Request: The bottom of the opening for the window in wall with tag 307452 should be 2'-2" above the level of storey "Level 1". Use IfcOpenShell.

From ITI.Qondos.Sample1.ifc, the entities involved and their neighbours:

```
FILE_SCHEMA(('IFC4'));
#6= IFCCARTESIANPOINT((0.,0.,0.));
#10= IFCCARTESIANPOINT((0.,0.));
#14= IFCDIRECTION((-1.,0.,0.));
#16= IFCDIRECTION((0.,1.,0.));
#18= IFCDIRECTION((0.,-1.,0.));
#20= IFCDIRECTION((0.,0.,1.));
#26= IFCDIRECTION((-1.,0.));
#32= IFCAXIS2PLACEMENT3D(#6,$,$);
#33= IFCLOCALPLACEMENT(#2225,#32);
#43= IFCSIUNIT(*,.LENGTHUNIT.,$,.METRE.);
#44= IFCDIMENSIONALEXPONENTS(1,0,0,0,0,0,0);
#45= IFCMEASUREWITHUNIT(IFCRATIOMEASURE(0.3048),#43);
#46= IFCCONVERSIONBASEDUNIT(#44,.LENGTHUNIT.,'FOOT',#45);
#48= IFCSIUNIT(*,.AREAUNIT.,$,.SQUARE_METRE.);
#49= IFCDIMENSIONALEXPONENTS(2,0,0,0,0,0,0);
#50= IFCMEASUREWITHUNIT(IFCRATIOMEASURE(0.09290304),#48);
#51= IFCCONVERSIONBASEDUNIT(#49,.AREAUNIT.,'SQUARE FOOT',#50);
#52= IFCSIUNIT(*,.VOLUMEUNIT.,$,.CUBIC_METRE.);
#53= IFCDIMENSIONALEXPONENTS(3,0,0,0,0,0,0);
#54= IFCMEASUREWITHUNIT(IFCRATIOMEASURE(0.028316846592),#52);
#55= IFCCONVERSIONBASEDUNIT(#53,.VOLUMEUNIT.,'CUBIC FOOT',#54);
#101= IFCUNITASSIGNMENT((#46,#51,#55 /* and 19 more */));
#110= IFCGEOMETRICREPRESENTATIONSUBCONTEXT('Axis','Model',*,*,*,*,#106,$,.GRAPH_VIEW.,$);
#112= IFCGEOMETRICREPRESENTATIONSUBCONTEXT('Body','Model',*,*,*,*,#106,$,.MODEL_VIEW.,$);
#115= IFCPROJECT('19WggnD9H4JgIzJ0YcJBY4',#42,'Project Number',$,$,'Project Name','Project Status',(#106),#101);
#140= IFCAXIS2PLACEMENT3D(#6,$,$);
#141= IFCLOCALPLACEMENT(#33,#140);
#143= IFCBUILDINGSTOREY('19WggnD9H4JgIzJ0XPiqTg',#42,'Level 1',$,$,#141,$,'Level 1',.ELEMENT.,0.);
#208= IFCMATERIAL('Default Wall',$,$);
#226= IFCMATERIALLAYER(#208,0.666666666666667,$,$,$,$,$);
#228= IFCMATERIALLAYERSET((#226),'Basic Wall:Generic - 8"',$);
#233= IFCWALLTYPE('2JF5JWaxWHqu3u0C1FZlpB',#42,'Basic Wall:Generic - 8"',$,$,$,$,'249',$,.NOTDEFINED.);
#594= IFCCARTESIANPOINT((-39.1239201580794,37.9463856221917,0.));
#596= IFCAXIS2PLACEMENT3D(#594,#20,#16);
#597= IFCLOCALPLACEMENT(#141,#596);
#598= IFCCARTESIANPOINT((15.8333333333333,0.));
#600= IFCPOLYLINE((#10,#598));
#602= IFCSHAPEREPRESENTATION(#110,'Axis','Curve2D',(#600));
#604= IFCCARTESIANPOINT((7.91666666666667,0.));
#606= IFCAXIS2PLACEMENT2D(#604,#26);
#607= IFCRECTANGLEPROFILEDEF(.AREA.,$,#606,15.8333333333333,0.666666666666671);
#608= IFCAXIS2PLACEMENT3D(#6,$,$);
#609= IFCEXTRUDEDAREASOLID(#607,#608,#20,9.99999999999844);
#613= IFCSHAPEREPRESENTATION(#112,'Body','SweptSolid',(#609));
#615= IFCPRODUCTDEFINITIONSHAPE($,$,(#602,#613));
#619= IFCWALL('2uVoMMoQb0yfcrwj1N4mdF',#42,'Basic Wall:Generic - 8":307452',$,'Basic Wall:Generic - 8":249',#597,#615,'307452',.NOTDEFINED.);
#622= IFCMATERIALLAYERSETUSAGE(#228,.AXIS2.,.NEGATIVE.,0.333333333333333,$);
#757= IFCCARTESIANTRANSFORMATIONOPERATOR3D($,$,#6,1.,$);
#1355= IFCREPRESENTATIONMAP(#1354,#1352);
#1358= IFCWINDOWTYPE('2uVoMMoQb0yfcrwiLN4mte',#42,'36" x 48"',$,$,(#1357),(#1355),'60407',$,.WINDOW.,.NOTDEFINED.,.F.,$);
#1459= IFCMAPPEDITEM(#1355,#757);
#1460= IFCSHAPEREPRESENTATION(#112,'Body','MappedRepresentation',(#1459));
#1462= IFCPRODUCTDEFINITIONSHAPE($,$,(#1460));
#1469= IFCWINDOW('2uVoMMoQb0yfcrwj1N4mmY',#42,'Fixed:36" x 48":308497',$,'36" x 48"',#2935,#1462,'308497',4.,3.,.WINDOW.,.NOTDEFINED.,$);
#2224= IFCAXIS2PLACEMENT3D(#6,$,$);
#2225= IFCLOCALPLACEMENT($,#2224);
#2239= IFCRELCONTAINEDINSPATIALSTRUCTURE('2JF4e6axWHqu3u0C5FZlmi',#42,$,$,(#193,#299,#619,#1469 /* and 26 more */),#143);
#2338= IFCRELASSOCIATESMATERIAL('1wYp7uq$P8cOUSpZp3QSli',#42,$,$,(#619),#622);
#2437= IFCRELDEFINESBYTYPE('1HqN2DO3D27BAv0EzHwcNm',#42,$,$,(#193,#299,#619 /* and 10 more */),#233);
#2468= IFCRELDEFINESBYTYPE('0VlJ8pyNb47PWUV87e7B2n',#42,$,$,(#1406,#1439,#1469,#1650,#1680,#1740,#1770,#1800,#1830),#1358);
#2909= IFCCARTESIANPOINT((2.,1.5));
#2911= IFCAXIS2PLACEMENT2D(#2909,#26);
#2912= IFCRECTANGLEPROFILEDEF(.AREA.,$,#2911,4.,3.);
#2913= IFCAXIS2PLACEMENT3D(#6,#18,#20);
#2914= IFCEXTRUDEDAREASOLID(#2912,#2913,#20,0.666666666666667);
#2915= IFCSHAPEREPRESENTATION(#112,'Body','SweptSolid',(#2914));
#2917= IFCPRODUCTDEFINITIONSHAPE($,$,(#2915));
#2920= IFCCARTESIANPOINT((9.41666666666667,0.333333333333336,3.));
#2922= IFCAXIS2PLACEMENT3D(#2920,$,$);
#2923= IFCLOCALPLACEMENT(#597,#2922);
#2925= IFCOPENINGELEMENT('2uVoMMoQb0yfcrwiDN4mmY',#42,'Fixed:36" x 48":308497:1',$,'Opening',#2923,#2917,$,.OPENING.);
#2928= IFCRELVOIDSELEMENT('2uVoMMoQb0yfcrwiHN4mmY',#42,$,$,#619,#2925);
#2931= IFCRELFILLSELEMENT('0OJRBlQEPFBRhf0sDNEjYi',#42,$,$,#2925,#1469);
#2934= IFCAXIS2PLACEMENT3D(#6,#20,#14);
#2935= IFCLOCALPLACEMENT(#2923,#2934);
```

```python
import numpy as np
import ifcopenshell
import ifcopenshell.api.geometry
import ifcopenshell.geom
import ifcopenshell.util.element
import ifcopenshell.util.placement
import ifcopenshell.util.shape
import ifcopenshell.util.unit

model = ifcopenshell.open("ITI.Qondos.Sample1.ifc")
unit_scale = ifcopenshell.util.unit.calculate_unit_scale(model)

window = model.by_id(1469)
opening = window.FillsVoids[0].RelatingOpeningElement
storey = ifcopenshell.util.element.get_container(window, ifc_class="IfcBuildingStorey")
level = ifcopenshell.util.placement.get_local_placement(storey.ObjectPlacement)[2, 3]

# The opening's origin need not be at the sill, so measure its lowest point.
shape = ifcopenshell.geom.create_shape(ifcopenshell.geom.settings(), opening)
bottom = ifcopenshell.util.shape.get_shape_bottom_elevation(shape, shape.geometry) / unit_scale
dz = level + 26 * 0.0254 / unit_scale - bottom

shift = np.array([0.0, 0.0, dz])
# The window is placed relative to its opening, so it follows when the opening moves.
matrix = ifcopenshell.util.placement.get_local_placement(opening.ObjectPlacement)
matrix[:3, 3] += shift
ifcopenshell.api.geometry.edit_object_placement(
    model, product=opening, matrix=matrix, is_si=False, should_transform_children=True
)

print(f"moved by {dz * unit_scale:+.3f} m")

model.write("ITI.Qondos.Sample1_v2.ifc")
```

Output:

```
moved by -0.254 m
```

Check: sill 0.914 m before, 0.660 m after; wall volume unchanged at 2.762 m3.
